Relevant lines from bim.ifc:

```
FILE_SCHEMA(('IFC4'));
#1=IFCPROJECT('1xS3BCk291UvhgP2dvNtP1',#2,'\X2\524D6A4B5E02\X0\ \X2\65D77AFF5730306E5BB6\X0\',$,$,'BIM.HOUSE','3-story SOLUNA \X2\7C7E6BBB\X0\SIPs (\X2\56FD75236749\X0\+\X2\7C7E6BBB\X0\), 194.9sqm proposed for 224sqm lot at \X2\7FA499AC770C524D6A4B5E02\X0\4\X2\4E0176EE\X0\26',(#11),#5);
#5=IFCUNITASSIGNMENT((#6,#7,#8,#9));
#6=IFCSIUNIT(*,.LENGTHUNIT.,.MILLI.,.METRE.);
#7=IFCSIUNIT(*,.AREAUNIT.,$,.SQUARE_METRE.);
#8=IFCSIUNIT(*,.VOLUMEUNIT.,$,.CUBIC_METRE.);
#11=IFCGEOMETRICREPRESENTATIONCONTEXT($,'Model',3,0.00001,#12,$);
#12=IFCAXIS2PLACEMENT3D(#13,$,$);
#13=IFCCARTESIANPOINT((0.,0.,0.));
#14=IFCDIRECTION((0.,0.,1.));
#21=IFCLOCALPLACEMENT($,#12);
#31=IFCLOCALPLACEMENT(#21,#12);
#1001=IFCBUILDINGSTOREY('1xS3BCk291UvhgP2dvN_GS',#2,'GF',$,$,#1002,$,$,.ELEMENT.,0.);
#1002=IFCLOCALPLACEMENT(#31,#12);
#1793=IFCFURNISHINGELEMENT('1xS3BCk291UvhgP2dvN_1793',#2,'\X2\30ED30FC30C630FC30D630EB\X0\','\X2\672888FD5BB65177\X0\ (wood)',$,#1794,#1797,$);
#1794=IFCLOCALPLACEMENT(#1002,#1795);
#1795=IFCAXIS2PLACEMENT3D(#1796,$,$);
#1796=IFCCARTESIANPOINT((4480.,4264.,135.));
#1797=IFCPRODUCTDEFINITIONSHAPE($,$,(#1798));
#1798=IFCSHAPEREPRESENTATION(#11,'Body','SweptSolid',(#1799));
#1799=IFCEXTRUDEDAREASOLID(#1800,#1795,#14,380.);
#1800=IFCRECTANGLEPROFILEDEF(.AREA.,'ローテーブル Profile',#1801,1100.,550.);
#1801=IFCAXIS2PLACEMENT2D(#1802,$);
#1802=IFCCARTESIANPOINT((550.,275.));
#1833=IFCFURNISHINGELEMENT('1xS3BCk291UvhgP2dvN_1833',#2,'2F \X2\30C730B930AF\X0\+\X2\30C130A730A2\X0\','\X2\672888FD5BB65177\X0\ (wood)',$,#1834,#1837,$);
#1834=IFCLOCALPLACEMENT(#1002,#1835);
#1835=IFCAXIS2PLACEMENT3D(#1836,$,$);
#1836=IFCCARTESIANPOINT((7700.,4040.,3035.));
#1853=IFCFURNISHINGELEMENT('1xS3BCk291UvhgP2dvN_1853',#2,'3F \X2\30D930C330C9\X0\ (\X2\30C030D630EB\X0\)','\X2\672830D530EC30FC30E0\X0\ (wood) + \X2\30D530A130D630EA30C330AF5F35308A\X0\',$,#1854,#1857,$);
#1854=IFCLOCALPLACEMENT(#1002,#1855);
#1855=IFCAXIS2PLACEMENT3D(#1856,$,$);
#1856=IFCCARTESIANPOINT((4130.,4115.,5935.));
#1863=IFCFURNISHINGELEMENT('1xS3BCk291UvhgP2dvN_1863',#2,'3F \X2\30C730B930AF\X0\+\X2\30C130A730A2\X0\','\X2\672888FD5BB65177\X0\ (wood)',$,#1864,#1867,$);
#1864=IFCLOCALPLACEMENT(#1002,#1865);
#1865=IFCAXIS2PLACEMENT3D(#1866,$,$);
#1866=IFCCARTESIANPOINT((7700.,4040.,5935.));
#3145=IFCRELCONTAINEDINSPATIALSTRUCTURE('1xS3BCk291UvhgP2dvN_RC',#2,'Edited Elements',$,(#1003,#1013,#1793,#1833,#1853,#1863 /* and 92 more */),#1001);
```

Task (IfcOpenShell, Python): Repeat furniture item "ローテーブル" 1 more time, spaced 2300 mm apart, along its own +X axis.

```python
import ifcopenshell
import ifcopenshell.api.geometry
import ifcopenshell.api.root
import ifcopenshell.util.element
import ifcopenshell.util.placement
import ifcopenshell.util.unit

model = ifcopenshell.open("bim.ifc")
unit_scale = ifcopenshell.util.unit.calculate_unit_scale(model)


def reuse_history(source, copy):
    """copy_class also copies each property set's owner history, people and application; keep the originals."""
    for rel in copy.IsDefinedBy:
        if rel.is_a("IfcRelDefinesByProperties") and (history := rel.RelatingPropertyDefinition.OwnerHistory):
            rel.RelatingPropertyDefinition.OwnerHistory = source.OwnerHistory
            ifcopenshell.util.element.remove_deep2(model, history)


source = model.by_guid("1xS3BCk291UvhgP2dvN_1793")
base = ifcopenshell.util.placement.get_local_placement(source.ObjectPlacement)
step = base[:3, 0] * 2.3 / unit_scale

for i in range(1, 2):
    copy = ifcopenshell.api.root.copy_class(model, product=source)
    copy.Representation = ifcopenshell.util.element.copy_deep(
        model, source.Representation, exclude=["IfcGeometricRepresentationContext", "IfcRepresentationMap"]
    )
    reuse_history(source, copy)
    matrix = base.copy()
    matrix[:3, 3] += i * step
    print("added at", matrix[:3, 3].round(3) + 0.0)
    ifcopenshell.api.geometry.edit_object_placement(model, product=copy, matrix=matrix, is_si=False)

model.write("bim_updated.ifc")
```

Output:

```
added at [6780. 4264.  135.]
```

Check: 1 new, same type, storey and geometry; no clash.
